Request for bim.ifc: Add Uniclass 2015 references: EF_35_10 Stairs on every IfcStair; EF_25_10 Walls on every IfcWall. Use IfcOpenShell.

First a look at what the model holds.

```python
import ifcopenshell

model = ifcopenshell.open("bim.ifc")
print(model.schema)
print("classifications:", [c.Name for c in model.by_type("IfcClassification")])
for ifc_class in ("IfcDoor", "IfcRoof", "IfcStair", "IfcWall", "IfcWindow"):
    print(ifc_class, len(model.by_type(ifc_class)))
```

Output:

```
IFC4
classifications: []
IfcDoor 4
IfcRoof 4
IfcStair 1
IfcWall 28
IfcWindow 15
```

```python
import ifcopenshell
import ifcopenshell.api.classification

model = ifcopenshell.open("bim.ifc")

system = ifcopenshell.api.classification.add_classification(model, classification="Uniclass 2015")

codes = {
    "IfcStair": ("EF_35_10", "Stairs"),
    "IfcWall": ("EF_25_10", "Walls"),
}
for ifc_class, (code, name) in codes.items():
    products = model.by_type(ifc_class)
    ifcopenshell.api.classification.add_reference(
        model, products=products, classification=system, identification=code, name=name
    )
    print(code, len(products))

model.write("bim_rev.ifc")
```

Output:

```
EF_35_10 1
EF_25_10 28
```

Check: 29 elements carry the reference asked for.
